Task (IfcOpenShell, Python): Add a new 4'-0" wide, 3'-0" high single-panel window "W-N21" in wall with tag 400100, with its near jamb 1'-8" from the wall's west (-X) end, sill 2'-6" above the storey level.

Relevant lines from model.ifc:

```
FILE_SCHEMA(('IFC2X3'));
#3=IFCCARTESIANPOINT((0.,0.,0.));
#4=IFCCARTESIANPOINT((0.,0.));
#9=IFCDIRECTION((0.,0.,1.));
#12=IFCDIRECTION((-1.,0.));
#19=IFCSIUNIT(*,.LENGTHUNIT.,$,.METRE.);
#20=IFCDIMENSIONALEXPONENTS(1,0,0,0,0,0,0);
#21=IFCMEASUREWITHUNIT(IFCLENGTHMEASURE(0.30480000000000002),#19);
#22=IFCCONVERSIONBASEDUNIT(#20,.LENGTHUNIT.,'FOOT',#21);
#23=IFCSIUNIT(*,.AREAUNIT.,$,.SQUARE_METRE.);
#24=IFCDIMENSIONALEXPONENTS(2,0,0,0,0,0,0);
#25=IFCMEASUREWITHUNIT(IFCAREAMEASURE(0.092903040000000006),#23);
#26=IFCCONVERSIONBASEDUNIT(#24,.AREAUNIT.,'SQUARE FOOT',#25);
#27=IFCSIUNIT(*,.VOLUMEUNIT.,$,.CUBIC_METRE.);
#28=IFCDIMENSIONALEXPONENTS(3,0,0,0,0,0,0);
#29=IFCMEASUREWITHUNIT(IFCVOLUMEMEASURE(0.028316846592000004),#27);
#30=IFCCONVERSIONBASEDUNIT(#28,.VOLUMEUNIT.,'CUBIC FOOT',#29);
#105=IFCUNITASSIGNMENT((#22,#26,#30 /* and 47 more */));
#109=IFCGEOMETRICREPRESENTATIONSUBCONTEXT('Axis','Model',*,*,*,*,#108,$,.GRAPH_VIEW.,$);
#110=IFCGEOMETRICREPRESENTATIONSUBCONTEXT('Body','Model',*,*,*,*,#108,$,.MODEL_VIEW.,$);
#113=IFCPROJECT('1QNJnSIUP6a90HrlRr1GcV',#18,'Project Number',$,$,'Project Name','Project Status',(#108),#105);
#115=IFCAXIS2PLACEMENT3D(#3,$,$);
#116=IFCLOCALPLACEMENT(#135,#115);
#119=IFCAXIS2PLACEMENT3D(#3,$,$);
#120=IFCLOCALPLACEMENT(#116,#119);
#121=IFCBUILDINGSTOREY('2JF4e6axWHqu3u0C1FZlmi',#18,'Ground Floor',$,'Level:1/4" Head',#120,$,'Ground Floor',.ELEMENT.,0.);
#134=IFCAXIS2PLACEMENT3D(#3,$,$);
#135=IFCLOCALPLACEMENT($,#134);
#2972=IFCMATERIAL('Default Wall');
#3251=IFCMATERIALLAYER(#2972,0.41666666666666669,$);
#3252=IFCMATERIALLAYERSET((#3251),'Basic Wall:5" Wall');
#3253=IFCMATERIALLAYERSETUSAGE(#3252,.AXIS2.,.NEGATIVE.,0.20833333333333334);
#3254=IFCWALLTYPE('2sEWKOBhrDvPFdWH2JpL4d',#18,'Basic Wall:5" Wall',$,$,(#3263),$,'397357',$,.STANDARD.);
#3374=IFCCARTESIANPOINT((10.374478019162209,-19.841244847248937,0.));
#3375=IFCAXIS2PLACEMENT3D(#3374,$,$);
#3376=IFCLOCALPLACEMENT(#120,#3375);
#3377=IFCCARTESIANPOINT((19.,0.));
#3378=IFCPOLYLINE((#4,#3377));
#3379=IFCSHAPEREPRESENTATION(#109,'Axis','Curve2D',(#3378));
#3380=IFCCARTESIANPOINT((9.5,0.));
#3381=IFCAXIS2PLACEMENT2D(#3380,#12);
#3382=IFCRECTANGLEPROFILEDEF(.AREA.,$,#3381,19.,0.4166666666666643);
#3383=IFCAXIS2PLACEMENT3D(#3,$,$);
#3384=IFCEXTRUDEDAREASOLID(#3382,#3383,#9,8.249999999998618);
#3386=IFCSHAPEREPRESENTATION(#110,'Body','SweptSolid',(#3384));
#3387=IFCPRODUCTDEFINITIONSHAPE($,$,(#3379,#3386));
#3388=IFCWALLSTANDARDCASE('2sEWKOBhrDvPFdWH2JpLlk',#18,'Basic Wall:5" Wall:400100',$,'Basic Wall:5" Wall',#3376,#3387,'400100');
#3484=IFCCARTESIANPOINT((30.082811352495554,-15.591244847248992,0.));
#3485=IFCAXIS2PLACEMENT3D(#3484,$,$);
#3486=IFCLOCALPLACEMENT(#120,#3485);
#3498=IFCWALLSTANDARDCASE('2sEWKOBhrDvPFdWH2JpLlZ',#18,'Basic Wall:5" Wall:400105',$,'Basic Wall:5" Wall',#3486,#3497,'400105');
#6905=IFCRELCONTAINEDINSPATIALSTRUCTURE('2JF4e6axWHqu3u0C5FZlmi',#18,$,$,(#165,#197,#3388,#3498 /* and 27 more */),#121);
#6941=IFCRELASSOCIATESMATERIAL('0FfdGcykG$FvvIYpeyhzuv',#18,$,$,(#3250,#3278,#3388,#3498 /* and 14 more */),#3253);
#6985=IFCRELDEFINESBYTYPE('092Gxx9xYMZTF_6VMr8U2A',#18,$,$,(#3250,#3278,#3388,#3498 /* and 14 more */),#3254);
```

```python
import numpy as np
import ifcopenshell
import ifcopenshell.api.feature
import ifcopenshell.api.geometry
import ifcopenshell.api.root
import ifcopenshell.api.spatial
import ifcopenshell.api.type
import ifcopenshell.geom
import ifcopenshell.util.element
import ifcopenshell.util.placement
import ifcopenshell.util.representation
import ifcopenshell.util.shape
import ifcopenshell.util.unit

model = ifcopenshell.open("model.ifc")
unit_scale = ifcopenshell.util.unit.calculate_unit_scale(model)
settings = ifcopenshell.geom.settings()


def volume(element):
    """Net volume in cubic metres, openings subtracted."""
    shape = ifcopenshell.geom.create_shape(settings, element)
    return ifcopenshell.util.shape.get_volume(shape.geometry)


wall = model.by_id(3388)
storey = ifcopenshell.util.element.get_container(wall, ifc_class="IfcBuildingStorey")
context = ifcopenshell.util.representation.get_context(model, "Model", "Body", "MODEL_VIEW")
before = volume(wall)

width, height, from_end, sill = 1.2192, 0.9144, 0.508, 0.762  # metres

# The wall runs along its own X axis, and the end named is its -X end.
wall_shape = ifcopenshell.geom.create_shape(settings, wall)
x, y, z = ifcopenshell.util.shape.get_vertices(wall_shape.geometry).T
start = x.min() + from_end
face, thickness = float(y.min()), float(y.max() - y.min())
wall_matrix = ifcopenshell.util.placement.get_local_placement(wall.ObjectPlacement)
level = ifcopenshell.util.placement.get_local_placement(storey.ObjectPlacement)[2, 3]


def in_wall(x, y):
    """Placement at x, y metres in the wall's axes, at sill height."""
    matrix = wall_matrix.copy()
    matrix[:, 3] = wall_matrix @ np.array([x / unit_scale, y / unit_scale, 0.0, 1.0])
    matrix[2, 3] = level + sill / unit_scale
    return matrix


# Opening: a box that overshoots both wall faces by 50 mm.
opening = ifcopenshell.api.root.create_entity(model, ifc_class="IfcOpeningElement")
box = ifcopenshell.api.geometry.add_wall_representation(
    model, context=context, length=width, height=height, thickness=thickness + 0.1
)
ifcopenshell.api.geometry.assign_representation(model, product=opening, representation=box)
ifcopenshell.api.geometry.edit_object_placement(model, product=opening, matrix=in_wall(start, face - 0.05), is_si=False)
ifcopenshell.api.feature.add_feature(model, feature=opening, element=wall)

window = ifcopenshell.api.root.create_entity(model, ifc_class="IfcWindow", name="W-N21")
window.OverallWidth, window.OverallHeight = width / unit_scale, height / unit_scale
body = ifcopenshell.api.geometry.add_window_representation(
    model,
    context=context,
    overall_width=window.OverallWidth,
    overall_height=window.OverallHeight,
    partition_type="SINGLE_PANEL",
)
ifcopenshell.api.geometry.assign_representation(model, product=window, representation=body)
ifcopenshell.api.spatial.assign_container(model, products=[window], relating_structure=storey)
fills = ifcopenshell.api.feature.add_filling(model, opening=opening, element=window)
fills.OwnerHistory = window.OwnerHistory  # required in IFC2X3

# IFC2X3 keeps the operation on the window style.
style = ifcopenshell.api.root.create_entity(model, ifc_class="IfcWindowStyle", name="W-N21")
style.OperationType, style.ConstructionType = "SINGLE_PANEL", "NOTDEFINED"
style.ParameterTakesPrecedence = style.Sizeable = False
ifcopenshell.api.type.assign_type(model, related_objects=[window], relating_type=style)

# Centre the window in the wall's thickness.
ifcopenshell.api.geometry.edit_object_placement(model, product=window, matrix=in_wall(start, face), is_si=False)
window_shape = ifcopenshell.geom.create_shape(settings, window)
depth = ifcopenshell.util.shape.get_vertices(window_shape.geometry)[:, 1]
offset = face + thickness / 2 - (depth.min() + depth.max()) / 2
ifcopenshell.api.geometry.edit_object_placement(model, product=window, matrix=in_wall(start, offset), is_si=False)

after = volume(wall)

print(f"wall volume {before:.3f} -> {after:.3f} m3")

model.write("model-out.ifc")
```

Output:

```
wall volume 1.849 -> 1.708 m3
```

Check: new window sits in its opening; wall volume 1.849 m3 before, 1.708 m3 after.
